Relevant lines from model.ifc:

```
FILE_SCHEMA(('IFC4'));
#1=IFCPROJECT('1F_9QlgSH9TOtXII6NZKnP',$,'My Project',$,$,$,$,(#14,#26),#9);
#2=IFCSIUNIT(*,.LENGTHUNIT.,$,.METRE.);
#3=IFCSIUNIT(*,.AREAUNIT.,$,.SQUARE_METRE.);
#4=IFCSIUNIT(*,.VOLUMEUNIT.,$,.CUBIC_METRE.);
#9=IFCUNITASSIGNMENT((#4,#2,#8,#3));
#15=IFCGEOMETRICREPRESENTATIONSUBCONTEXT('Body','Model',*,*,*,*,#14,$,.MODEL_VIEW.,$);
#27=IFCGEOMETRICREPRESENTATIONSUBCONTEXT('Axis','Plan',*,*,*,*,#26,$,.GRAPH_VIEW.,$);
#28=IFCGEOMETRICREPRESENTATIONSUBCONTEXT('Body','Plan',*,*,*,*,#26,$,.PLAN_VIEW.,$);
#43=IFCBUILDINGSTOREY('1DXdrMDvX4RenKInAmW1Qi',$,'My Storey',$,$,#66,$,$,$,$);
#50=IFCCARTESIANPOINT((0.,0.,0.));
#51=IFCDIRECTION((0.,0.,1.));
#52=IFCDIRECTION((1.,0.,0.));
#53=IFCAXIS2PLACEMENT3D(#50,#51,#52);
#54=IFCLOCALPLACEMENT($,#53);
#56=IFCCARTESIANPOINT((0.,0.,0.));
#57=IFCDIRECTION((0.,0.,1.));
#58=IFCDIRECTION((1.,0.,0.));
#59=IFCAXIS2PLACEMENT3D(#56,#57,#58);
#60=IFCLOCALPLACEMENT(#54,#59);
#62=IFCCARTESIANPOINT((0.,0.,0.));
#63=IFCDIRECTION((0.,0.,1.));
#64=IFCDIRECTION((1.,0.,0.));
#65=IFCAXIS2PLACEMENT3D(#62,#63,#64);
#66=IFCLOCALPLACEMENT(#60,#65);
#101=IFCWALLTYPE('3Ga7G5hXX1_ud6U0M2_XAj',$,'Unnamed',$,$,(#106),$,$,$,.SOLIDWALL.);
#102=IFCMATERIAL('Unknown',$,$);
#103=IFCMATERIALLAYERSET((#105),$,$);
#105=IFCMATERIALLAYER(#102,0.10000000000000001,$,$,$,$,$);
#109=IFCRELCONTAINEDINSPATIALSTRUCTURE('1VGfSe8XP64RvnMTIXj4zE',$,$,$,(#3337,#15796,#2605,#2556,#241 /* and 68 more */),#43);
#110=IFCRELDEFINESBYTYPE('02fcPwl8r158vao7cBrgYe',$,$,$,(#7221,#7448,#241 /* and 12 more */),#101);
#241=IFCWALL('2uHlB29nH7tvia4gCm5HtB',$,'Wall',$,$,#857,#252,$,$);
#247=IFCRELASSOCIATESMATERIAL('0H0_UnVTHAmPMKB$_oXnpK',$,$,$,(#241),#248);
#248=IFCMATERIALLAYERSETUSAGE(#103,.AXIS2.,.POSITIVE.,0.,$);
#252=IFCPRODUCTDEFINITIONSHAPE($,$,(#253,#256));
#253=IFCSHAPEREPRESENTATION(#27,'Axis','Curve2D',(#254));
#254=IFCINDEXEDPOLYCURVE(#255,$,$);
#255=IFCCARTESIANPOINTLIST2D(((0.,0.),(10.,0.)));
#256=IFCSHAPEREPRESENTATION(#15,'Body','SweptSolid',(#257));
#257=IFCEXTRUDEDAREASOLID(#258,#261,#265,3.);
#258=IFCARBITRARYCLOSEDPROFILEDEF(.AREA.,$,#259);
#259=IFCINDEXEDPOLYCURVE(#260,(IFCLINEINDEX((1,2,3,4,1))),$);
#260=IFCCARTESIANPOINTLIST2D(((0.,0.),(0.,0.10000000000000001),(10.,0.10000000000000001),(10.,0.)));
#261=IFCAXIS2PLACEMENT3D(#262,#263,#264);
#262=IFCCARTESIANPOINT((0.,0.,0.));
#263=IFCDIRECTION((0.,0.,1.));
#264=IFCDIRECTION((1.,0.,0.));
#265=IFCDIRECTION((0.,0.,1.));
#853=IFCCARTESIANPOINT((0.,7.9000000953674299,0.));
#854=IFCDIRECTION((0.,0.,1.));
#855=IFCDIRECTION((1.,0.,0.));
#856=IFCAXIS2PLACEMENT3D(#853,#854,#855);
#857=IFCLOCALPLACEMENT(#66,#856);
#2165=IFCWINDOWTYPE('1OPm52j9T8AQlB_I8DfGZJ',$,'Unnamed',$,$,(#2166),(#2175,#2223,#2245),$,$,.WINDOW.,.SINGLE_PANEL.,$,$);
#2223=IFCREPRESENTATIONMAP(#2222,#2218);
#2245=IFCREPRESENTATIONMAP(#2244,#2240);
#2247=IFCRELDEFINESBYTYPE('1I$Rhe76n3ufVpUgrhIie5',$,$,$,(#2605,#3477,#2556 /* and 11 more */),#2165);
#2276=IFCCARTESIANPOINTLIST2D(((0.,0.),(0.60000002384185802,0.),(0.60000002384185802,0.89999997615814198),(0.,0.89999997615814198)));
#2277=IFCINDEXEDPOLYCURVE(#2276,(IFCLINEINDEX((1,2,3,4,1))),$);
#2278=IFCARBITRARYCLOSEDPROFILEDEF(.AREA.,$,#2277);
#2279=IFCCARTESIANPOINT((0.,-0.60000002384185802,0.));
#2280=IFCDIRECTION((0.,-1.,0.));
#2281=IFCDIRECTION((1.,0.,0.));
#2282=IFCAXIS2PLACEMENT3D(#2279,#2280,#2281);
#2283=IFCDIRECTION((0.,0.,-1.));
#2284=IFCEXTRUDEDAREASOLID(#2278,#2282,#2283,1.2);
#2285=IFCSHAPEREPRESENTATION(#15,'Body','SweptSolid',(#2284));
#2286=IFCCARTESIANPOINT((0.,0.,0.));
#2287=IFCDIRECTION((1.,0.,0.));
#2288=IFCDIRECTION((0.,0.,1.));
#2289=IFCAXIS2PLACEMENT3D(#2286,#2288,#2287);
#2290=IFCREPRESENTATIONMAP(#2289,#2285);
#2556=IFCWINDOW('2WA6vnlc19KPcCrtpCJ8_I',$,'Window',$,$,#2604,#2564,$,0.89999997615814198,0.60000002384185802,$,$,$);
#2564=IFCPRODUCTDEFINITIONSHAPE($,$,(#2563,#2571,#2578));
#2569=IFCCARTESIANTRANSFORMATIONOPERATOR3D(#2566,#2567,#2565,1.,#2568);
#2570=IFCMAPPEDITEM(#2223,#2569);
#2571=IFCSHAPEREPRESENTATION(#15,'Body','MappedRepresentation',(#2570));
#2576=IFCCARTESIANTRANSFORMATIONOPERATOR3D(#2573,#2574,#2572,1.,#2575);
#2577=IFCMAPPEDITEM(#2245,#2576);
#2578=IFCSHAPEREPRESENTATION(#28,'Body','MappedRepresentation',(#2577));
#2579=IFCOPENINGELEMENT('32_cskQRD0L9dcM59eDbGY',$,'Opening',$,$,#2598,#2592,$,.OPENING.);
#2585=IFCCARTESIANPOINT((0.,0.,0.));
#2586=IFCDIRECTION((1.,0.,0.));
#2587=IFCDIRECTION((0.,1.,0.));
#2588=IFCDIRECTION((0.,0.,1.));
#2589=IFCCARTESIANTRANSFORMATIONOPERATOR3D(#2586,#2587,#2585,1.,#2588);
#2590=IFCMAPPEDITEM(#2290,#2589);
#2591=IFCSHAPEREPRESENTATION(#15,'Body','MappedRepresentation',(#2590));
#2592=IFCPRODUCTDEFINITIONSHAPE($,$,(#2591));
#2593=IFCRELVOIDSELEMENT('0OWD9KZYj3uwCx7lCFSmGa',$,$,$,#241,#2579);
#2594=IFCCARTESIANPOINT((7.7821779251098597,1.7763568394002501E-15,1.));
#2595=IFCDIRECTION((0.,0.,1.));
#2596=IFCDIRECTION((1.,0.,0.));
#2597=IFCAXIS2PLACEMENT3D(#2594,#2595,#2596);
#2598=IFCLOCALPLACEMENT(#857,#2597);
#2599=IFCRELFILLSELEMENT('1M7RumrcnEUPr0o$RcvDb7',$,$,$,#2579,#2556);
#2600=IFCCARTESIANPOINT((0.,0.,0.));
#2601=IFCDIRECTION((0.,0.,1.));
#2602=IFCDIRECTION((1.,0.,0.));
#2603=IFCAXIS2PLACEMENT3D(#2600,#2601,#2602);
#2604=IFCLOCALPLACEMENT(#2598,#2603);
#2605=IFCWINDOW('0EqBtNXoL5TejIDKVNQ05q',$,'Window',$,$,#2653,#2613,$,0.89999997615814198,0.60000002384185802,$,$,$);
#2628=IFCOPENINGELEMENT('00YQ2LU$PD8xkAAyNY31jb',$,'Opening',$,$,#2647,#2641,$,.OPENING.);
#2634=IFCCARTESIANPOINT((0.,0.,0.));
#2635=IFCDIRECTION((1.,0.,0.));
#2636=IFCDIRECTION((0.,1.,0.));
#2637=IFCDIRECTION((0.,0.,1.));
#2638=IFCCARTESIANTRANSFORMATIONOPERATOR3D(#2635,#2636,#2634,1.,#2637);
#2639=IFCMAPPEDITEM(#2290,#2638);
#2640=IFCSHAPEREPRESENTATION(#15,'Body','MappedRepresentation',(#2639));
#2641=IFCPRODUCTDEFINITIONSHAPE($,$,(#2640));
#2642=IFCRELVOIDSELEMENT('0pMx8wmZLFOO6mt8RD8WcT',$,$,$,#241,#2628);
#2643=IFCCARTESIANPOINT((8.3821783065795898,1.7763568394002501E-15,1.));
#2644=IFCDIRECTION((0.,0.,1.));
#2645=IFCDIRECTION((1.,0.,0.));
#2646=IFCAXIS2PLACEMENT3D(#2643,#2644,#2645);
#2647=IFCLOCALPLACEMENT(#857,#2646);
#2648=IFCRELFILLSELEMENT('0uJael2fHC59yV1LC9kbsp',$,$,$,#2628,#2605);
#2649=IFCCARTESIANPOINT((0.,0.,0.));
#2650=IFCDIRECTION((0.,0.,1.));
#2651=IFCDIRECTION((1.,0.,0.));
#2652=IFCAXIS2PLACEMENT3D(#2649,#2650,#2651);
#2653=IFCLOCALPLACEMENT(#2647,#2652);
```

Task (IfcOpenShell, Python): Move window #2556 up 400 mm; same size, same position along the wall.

```python
import numpy as np
import ifcopenshell
import ifcopenshell.api.geometry
import ifcopenshell.util.placement
import ifcopenshell.util.unit

model = ifcopenshell.open("model.ifc")
unit_scale = ifcopenshell.util.unit.calculate_unit_scale(model)

window = model.by_id(2556)
opening = window.FillsVoids[0].RelatingOpeningElement
dz = 0.4

shift = np.array([0.0, 0.0, dz])
# The window is placed relative to its opening, so it follows when the opening moves.
matrix = ifcopenshell.util.placement.get_local_placement(opening.ObjectPlacement)
matrix[:3, 3] += shift
ifcopenshell.api.geometry.edit_object_placement(
    model, product=opening, matrix=matrix, is_si=False, should_transform_children=True
)

print(f"moved by {dz * unit_scale:+.3f} m")

model.write("model_v2.ifc")
```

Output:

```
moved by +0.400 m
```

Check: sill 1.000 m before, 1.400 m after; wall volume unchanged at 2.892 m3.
